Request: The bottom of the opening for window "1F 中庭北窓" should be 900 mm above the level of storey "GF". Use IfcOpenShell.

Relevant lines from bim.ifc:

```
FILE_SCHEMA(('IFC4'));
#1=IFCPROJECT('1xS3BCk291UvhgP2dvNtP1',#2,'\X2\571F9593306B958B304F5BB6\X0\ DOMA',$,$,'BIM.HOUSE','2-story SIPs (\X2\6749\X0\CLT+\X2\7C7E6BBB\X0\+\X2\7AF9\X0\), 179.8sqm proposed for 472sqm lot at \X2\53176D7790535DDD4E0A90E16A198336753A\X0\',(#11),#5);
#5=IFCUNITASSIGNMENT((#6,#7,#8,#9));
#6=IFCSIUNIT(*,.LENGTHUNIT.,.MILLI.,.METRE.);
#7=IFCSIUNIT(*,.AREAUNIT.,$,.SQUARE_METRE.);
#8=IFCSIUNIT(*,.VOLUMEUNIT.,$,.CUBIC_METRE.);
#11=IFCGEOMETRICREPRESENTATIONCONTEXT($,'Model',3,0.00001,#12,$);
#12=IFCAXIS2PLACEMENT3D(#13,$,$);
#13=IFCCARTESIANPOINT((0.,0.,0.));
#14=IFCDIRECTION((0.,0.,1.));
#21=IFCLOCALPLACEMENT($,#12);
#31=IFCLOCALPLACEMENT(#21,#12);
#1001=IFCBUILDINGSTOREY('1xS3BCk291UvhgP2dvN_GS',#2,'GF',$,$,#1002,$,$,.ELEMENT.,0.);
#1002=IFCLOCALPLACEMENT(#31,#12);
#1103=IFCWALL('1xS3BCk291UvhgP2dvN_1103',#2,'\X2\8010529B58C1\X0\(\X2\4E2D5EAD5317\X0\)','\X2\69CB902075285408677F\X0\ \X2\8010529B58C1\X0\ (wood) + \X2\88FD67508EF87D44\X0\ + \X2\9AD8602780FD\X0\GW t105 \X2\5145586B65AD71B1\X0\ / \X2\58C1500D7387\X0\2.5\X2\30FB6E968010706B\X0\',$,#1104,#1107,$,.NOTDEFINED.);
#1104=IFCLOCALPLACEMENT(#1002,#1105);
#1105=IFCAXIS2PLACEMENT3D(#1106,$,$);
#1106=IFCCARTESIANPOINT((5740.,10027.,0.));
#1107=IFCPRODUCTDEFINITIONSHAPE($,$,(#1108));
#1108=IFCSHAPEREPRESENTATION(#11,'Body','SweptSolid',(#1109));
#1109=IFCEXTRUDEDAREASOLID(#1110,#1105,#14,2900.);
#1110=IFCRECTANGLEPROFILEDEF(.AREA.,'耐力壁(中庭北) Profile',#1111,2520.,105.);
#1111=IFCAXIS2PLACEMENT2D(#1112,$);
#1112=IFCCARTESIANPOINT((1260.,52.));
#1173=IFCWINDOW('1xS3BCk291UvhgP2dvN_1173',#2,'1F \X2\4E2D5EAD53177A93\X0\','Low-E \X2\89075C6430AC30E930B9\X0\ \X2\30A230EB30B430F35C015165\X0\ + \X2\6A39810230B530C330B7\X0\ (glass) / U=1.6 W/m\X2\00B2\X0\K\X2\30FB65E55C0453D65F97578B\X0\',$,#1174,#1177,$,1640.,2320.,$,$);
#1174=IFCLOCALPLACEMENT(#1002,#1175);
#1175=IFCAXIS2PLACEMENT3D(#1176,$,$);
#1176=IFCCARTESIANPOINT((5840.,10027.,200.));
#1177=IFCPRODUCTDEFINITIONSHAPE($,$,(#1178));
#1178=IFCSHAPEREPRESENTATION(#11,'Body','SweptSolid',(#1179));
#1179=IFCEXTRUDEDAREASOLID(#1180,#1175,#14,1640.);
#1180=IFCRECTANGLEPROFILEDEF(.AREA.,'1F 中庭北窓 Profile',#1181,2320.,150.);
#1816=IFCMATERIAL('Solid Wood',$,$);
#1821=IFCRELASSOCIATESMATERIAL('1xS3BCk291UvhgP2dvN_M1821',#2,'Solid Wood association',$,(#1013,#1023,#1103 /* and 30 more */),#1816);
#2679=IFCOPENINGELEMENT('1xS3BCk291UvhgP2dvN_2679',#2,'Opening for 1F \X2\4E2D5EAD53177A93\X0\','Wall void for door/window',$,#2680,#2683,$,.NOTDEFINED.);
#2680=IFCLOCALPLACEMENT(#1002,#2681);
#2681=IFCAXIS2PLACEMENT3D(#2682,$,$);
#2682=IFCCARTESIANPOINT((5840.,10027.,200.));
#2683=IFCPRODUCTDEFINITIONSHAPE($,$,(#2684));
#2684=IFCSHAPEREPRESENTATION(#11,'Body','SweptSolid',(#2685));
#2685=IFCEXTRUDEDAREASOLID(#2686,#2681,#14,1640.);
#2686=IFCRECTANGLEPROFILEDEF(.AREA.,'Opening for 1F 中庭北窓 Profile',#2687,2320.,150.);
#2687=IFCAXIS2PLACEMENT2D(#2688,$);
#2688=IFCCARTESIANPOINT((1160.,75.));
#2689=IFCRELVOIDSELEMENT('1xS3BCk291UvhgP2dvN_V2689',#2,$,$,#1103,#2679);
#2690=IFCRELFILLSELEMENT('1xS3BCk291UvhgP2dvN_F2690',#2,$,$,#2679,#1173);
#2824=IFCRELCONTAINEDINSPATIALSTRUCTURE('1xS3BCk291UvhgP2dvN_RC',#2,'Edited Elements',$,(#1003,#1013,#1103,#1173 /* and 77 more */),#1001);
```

```python
import numpy as np
import ifcopenshell
import ifcopenshell.api.geometry
import ifcopenshell.geom
import ifcopenshell.util.element
import ifcopenshell.util.placement
import ifcopenshell.util.shape
import ifcopenshell.util.unit

model = ifcopenshell.open("bim.ifc")
unit_scale = ifcopenshell.util.unit.calculate_unit_scale(model)

window = model.by_id(1173)
opening = window.FillsVoids[0].RelatingOpeningElement
storey = ifcopenshell.util.element.get_container(window, ifc_class="IfcBuildingStorey")
level = ifcopenshell.util.placement.get_local_placement(storey.ObjectPlacement)[2, 3]

# The opening's origin need not be at the sill, so measure its lowest point.
shape = ifcopenshell.geom.create_shape(ifcopenshell.geom.settings(), opening)
bottom = ifcopenshell.util.shape.get_shape_bottom_elevation(shape, shape.geometry) / unit_scale
dz = level + 0.9 / unit_scale - bottom

shift = np.array([0.0, 0.0, dz])
# The window is not placed relative to its opening, so move both.
for product in (opening, window):
    matrix = ifcopenshell.util.placement.get_local_placement(product.ObjectPlacement)
    matrix[:3, 3] += shift
    ifcopenshell.api.geometry.edit_object_placement(model, product=product, matrix=matrix, is_si=False)

print(f"moved by {dz * unit_scale:+.3f} m")

model.write("bim_updated.ifc")
```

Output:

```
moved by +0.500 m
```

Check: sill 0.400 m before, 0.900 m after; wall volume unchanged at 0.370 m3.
